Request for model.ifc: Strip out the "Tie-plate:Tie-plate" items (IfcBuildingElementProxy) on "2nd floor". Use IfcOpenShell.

First a look at what the model holds.

```python
import ifcopenshell
import ifcopenshell.util.element

model = ifcopenshell.open("model.ifc")
print(model.schema)
storey = next(s for s in model.by_type("IfcBuildingStorey") if s.Name == "2nd floor")
proxies = [e for e in ifcopenshell.util.element.get_decomposition(storey) if e.is_a("IfcBuildingElementProxy")]
seen = {}
for e in proxies:
    element_type = ifcopenshell.util.element.get_type(e)
    name = element_type.Name if element_type not in (None, e) else None
    seen[name] = seen.get(name, 0) + 1
for name, count in sorted(seen.items(), key=str):
    print(count, "x", name)
```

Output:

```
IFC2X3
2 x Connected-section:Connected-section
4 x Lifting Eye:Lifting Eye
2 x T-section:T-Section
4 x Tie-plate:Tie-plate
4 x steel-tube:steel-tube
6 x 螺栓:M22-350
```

```python
import ifcopenshell
import ifcopenshell.api.root
import ifcopenshell.util.element

model = ifcopenshell.open("model.ifc")

storey = next(s for s in model.by_type("IfcBuildingStorey") if s.Name == "2nd floor")
proxies = [e for e in ifcopenshell.util.element.get_decomposition(storey) if e.is_a("IfcBuildingElementProxy")]
targets = [e for e in proxies if (t := ifcopenshell.util.element.get_type(e)) not in (None, e) and t.Name == "Tie-plate:Tie-plate"]

for e in targets:
    ifcopenshell.api.root.remove_product(model, product=e)
print(len(targets), "removed")

model.write("model_edited.ifc")
```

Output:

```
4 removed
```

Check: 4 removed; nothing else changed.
